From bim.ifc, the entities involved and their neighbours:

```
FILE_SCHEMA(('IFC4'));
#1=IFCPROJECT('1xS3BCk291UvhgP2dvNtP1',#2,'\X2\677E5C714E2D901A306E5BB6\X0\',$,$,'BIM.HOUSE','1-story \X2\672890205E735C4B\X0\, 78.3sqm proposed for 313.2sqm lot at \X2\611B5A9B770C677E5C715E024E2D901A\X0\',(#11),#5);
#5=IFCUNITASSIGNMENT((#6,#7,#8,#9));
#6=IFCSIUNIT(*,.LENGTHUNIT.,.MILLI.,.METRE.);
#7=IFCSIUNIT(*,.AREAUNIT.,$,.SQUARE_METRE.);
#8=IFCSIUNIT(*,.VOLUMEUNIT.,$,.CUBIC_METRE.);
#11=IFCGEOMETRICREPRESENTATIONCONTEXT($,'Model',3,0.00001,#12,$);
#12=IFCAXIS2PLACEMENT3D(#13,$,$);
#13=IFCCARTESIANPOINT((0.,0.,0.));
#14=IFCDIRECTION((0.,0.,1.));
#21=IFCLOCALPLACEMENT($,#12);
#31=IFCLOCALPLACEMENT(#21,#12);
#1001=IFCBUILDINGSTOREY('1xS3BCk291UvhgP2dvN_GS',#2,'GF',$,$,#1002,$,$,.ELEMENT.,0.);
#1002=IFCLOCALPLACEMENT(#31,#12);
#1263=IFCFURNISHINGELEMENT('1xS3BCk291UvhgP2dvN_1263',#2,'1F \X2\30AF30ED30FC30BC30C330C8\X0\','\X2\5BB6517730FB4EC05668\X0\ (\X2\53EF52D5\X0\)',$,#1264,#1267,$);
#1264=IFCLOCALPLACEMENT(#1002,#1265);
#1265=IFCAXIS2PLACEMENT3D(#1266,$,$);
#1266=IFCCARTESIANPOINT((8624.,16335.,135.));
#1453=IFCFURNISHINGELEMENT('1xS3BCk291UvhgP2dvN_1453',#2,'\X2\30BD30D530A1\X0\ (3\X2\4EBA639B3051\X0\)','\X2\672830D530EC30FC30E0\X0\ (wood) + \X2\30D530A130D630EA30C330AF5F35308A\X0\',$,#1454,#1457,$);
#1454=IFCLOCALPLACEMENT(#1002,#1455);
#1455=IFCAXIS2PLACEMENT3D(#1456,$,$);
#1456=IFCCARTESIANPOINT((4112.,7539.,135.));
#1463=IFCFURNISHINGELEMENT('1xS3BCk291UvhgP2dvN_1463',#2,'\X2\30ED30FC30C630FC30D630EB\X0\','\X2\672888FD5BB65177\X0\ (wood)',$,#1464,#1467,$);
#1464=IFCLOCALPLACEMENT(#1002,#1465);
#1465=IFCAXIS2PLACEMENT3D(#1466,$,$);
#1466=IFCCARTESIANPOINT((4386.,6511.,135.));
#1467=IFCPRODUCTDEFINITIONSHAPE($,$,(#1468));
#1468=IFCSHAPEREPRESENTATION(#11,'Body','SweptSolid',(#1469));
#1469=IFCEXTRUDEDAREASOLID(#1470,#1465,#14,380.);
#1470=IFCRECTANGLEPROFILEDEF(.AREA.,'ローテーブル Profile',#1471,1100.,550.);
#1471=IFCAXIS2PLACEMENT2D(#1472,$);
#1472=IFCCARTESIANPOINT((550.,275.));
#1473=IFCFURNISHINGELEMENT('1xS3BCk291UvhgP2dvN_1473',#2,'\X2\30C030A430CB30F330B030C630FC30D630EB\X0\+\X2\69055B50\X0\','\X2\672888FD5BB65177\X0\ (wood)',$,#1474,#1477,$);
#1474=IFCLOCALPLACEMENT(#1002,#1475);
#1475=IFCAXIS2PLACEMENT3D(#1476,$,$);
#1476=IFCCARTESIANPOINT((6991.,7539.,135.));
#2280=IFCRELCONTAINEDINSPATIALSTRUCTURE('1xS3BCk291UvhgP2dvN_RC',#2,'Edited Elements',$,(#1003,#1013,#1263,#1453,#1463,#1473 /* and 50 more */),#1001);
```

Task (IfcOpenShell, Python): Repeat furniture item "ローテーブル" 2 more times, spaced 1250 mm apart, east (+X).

```python
import numpy as np
import ifcopenshell
import ifcopenshell.api.geometry
import ifcopenshell.api.root
import ifcopenshell.util.element
import ifcopenshell.util.placement
import ifcopenshell.util.unit

model = ifcopenshell.open("bim.ifc")
unit_scale = ifcopenshell.util.unit.calculate_unit_scale(model)


def reuse_history(source, copy):
    """copy_class also copies each property set's owner history, people and application; keep the originals."""
    for rel in copy.IsDefinedBy:
        if rel.is_a("IfcRelDefinesByProperties") and (history := rel.RelatingPropertyDefinition.OwnerHistory):
            rel.RelatingPropertyDefinition.OwnerHistory = source.OwnerHistory
            ifcopenshell.util.element.remove_deep2(model, history)


source = model.by_guid("1xS3BCk291UvhgP2dvN_1463")
base = ifcopenshell.util.placement.get_local_placement(source.ObjectPlacement)
step = np.array([1.0, 0.0, 0.0]) * 1.25 / unit_scale

for i in range(1, 3):
    copy = ifcopenshell.api.root.copy_class(model, product=source)
    copy.Representation = ifcopenshell.util.element.copy_deep(
        model, source.Representation, exclude=["IfcGeometricRepresentationContext", "IfcRepresentationMap"]
    )
    reuse_history(source, copy)
    matrix = base.copy()
    matrix[:3, 3] += i * step
    print("added at", matrix[:3, 3].round(3) + 0.0)
    ifcopenshell.api.geometry.edit_object_placement(model, product=copy, matrix=matrix, is_si=False)

model.write("bim_v2.ifc")
```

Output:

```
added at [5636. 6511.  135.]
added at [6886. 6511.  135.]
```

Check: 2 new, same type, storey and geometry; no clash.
